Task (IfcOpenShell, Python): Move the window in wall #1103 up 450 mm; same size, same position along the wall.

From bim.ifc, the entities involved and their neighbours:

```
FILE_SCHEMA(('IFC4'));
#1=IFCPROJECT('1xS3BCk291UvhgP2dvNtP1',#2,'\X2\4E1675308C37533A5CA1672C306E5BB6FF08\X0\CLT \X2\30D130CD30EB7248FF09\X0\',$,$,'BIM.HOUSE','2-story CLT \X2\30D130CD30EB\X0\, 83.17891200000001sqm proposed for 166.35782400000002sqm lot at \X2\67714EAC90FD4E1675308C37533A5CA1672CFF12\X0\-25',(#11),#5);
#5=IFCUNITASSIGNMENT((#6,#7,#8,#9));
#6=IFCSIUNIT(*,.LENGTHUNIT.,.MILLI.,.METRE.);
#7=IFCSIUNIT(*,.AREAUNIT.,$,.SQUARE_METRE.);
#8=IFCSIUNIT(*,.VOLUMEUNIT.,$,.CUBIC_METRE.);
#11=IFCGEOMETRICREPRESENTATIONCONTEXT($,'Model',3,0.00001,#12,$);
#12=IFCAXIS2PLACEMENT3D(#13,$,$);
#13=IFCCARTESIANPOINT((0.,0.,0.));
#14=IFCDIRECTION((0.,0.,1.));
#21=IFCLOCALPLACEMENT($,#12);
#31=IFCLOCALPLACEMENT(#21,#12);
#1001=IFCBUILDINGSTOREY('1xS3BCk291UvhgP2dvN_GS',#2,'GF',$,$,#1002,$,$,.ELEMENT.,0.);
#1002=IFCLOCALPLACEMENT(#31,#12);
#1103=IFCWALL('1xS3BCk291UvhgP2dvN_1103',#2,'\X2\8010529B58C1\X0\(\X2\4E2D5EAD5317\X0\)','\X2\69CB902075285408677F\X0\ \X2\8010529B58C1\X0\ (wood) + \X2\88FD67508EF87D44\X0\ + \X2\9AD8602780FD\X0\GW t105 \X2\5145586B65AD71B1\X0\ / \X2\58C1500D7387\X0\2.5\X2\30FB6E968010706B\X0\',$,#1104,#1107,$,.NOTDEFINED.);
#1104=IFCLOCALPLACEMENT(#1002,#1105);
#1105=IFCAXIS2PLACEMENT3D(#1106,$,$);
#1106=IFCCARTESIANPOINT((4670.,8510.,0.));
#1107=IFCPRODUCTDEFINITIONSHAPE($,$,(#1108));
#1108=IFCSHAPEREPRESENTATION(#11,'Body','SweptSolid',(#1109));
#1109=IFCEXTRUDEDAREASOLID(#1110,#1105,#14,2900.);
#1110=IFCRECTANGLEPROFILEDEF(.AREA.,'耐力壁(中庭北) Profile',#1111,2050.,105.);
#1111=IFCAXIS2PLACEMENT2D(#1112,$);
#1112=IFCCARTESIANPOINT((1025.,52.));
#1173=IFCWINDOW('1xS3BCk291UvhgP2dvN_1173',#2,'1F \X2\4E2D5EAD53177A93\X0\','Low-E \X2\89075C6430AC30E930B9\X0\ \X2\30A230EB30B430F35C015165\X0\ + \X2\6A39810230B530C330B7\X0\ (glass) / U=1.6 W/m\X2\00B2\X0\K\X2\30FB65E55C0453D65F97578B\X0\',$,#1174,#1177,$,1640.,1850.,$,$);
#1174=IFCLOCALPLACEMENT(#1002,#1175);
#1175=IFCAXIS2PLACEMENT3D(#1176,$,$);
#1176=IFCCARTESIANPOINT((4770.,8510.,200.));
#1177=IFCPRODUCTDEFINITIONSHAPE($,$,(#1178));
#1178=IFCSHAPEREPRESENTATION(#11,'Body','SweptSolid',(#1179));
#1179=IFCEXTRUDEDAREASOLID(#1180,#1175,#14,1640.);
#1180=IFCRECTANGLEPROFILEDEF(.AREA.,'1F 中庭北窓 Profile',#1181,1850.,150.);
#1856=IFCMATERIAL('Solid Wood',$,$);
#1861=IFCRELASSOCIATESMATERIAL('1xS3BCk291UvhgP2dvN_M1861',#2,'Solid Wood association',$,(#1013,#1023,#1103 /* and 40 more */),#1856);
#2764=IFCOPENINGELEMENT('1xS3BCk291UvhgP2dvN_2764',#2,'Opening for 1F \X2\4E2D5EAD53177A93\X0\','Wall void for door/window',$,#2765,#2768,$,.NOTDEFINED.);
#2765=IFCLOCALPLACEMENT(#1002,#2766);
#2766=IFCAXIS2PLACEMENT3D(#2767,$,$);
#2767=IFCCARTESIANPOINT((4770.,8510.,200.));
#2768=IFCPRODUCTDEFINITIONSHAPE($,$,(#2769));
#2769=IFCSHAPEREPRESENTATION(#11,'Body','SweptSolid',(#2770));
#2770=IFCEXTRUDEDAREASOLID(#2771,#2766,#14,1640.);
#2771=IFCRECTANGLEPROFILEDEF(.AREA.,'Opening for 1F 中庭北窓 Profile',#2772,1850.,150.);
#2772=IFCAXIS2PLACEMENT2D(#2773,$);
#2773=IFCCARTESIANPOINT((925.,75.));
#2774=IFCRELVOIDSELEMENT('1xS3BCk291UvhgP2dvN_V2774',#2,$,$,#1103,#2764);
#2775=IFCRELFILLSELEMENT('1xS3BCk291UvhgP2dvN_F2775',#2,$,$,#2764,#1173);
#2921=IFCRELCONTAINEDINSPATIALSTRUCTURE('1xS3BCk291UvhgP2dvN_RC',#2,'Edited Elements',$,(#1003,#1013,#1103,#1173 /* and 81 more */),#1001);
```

```python
import numpy as np
import ifcopenshell
import ifcopenshell.api.geometry
import ifcopenshell.util.placement
import ifcopenshell.util.unit

model = ifcopenshell.open("bim.ifc")
unit_scale = ifcopenshell.util.unit.calculate_unit_scale(model)

window = model.by_guid("1xS3BCk291UvhgP2dvN_1173")
opening = window.FillsVoids[0].RelatingOpeningElement
dz = 450.0

shift = np.array([0.0, 0.0, dz])
# The window is not placed relative to its opening, so move both.
for product in (opening, window):
    matrix = ifcopenshell.util.placement.get_local_placement(product.ObjectPlacement)
    matrix[:3, 3] += shift
    ifcopenshell.api.geometry.edit_object_placement(model, product=product, matrix=matrix, is_si=False)

print(f"moved by {dz * unit_scale:+.3f} m")

model.write("bim_rev.ifc")
```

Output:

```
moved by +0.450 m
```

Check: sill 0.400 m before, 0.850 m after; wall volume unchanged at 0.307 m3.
